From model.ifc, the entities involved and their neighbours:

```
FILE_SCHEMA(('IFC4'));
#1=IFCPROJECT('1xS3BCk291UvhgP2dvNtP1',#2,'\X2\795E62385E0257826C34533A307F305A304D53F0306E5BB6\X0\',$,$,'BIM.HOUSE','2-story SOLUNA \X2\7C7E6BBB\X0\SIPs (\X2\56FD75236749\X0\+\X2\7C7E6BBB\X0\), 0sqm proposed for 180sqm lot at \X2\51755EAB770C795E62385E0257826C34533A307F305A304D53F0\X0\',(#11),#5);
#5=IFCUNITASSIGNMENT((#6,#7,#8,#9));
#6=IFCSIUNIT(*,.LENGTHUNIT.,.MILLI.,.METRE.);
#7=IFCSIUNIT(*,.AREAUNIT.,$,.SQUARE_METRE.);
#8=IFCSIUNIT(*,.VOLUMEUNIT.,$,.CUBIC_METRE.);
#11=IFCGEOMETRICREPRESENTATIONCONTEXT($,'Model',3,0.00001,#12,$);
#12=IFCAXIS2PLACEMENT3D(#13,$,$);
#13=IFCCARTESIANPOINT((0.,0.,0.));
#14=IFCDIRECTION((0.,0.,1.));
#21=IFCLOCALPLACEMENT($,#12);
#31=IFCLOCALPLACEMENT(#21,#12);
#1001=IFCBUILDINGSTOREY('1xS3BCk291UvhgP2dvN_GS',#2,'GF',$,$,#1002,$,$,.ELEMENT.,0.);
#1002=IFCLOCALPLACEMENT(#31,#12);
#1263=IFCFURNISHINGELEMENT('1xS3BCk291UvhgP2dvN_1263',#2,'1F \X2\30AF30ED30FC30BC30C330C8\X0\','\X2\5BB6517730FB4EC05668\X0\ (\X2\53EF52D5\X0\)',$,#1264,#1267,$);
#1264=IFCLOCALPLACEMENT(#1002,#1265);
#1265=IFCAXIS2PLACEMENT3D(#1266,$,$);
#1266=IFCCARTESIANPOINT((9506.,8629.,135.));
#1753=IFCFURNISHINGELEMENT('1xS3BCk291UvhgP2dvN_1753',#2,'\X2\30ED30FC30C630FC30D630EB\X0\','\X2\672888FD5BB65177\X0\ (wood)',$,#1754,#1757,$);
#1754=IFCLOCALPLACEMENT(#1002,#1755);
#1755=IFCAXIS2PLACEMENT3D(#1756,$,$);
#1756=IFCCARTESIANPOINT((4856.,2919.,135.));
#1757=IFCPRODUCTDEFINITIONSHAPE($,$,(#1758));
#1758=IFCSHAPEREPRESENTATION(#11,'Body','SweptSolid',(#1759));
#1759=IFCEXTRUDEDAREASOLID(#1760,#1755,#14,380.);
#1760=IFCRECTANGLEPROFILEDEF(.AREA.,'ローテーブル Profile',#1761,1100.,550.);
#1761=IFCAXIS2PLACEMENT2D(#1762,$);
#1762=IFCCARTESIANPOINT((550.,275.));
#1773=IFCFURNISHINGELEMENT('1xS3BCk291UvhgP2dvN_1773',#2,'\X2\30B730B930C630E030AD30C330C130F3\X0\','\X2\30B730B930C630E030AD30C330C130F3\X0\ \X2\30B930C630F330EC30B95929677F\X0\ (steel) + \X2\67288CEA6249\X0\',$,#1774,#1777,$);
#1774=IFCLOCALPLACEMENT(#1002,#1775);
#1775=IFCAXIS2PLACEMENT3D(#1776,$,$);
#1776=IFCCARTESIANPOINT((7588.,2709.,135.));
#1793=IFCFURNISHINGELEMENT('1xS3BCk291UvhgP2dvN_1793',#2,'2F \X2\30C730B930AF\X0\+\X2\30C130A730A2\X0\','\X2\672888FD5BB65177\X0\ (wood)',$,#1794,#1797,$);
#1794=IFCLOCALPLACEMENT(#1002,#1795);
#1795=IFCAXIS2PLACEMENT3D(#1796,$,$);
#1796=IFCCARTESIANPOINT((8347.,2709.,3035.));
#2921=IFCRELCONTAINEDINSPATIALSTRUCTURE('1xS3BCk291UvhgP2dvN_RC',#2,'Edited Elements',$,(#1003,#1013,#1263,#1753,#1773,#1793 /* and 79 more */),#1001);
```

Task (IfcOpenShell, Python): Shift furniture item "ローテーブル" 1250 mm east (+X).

```python
import ifcopenshell
import ifcopenshell.api.geometry
import ifcopenshell.util.placement
import ifcopenshell.util.unit

model = ifcopenshell.open("model.ifc")
unit_scale = ifcopenshell.util.unit.calculate_unit_scale(model)

item = model.by_guid("1xS3BCk291UvhgP2dvN_1753")
matrix = ifcopenshell.util.placement.get_local_placement(item.ObjectPlacement)
matrix[0, 3] += 1.25 / unit_scale
ifcopenshell.api.geometry.edit_object_placement(model, product=item, matrix=matrix, is_si=False)

print(ifcopenshell.util.placement.get_local_placement(item.ObjectPlacement).round(3) + 0.0)

model.write("model_updated.ifc")
```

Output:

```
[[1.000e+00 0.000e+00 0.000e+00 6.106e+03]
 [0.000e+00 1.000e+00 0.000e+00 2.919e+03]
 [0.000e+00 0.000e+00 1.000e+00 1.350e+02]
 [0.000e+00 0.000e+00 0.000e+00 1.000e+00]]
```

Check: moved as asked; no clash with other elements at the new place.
